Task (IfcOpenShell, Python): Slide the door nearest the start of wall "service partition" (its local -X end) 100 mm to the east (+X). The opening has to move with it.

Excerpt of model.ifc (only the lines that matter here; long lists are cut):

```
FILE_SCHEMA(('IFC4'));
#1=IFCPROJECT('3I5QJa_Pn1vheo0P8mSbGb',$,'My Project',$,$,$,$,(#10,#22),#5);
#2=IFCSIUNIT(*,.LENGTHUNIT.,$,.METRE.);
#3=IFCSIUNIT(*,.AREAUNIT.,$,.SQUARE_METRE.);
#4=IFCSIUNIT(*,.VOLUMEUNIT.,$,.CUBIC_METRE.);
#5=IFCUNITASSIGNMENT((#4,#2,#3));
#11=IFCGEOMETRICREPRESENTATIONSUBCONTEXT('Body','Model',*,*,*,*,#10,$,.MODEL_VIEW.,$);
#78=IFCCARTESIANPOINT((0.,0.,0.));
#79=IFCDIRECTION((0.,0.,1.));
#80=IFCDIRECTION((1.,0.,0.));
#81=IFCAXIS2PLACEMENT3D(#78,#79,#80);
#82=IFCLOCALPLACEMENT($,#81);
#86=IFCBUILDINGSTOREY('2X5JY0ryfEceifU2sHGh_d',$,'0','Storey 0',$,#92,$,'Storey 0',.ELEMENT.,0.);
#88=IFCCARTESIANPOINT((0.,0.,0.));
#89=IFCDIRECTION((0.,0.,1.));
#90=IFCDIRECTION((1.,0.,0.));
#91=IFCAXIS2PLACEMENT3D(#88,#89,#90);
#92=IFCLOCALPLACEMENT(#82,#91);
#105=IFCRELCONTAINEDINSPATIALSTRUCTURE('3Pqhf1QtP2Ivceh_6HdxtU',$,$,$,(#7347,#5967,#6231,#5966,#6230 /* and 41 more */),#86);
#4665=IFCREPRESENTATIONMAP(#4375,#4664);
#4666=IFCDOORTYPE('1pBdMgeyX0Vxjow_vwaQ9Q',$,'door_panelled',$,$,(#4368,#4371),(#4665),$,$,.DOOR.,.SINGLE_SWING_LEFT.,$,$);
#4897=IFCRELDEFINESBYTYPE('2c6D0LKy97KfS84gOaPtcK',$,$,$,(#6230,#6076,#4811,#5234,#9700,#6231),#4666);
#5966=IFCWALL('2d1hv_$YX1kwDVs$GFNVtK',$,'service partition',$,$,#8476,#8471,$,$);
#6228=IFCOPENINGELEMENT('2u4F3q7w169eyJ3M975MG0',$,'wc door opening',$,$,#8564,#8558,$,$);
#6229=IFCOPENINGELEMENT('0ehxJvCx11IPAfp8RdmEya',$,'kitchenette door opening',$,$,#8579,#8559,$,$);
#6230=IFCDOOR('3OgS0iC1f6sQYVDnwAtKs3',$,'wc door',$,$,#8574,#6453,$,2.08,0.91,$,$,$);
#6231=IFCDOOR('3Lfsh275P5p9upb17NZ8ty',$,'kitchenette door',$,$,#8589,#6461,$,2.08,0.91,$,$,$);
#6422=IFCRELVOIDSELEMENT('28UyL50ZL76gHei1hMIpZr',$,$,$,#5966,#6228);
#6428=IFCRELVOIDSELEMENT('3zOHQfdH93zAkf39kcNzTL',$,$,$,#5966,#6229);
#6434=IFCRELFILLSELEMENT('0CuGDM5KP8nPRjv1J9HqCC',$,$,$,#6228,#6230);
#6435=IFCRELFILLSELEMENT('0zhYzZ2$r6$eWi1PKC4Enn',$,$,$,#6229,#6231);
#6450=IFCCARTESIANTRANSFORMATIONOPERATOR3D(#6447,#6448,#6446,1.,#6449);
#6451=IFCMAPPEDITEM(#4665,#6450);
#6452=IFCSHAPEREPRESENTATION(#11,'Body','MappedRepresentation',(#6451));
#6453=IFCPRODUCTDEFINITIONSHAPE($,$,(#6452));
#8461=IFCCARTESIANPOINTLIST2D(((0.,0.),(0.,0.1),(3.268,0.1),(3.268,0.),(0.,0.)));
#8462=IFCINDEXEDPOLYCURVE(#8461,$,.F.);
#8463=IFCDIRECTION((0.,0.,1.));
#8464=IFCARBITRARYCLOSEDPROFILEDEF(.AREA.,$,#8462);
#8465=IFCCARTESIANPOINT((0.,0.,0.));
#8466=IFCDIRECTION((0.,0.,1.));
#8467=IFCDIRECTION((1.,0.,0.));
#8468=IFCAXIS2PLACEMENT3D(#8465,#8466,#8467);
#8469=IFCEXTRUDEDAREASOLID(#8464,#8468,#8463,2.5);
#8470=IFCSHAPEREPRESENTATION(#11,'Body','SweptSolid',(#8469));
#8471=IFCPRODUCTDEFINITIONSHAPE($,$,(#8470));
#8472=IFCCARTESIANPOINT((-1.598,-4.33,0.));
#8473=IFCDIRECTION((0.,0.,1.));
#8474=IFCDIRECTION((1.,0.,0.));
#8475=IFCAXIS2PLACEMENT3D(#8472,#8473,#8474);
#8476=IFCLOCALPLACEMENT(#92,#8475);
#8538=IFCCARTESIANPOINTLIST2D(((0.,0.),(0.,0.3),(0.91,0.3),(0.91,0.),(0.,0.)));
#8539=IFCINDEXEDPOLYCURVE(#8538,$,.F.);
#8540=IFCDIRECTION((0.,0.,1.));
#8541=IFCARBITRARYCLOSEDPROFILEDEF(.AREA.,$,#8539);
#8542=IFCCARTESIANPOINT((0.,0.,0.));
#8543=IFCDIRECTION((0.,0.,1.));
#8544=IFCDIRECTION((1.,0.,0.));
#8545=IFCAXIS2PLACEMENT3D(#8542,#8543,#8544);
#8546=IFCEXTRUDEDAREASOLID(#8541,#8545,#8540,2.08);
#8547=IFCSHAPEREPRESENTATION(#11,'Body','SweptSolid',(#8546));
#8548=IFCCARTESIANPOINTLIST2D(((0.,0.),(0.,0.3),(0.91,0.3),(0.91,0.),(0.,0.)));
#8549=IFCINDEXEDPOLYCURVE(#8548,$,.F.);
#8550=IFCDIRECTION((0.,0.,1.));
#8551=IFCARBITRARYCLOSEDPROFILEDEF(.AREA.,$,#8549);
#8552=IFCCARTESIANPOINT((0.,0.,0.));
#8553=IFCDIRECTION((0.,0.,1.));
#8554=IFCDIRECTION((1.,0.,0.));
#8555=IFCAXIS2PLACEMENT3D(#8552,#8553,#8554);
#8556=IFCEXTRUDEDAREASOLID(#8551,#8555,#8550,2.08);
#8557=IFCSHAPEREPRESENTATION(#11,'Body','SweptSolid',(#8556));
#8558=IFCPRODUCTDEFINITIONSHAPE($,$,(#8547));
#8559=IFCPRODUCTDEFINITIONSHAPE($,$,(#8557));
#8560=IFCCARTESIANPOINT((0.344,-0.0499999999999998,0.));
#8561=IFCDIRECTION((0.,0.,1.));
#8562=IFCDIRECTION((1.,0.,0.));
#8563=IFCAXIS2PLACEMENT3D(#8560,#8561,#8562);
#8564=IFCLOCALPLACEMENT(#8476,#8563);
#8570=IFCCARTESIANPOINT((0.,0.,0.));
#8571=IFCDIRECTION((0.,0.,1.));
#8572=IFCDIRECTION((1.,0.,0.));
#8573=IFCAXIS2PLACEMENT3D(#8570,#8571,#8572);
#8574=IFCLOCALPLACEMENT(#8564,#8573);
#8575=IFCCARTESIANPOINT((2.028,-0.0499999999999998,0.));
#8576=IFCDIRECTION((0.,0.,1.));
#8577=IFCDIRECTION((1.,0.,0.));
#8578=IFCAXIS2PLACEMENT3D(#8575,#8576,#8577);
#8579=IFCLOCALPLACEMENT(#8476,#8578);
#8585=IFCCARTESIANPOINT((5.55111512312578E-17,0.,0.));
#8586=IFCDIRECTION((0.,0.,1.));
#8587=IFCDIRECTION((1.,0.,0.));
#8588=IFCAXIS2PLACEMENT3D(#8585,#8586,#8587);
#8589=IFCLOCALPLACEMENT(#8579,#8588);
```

```python
import ifcopenshell
import ifcopenshell.api.geometry
import ifcopenshell.util.placement
import ifcopenshell.util.unit

model = ifcopenshell.open("model.ifc")
unit_scale = ifcopenshell.util.unit.calculate_unit_scale(model)

door = model.by_guid("3OgS0iC1f6sQYVDnwAtKs3")
opening = door.FillsVoids[0].RelatingOpeningElement
wall = opening.VoidsElements[0].RelatingBuildingElement

wall_matrix = ifcopenshell.util.placement.get_local_placement(wall.ObjectPlacement)
shift = wall_matrix[:3, 0] * 0.1 / unit_scale
before = ifcopenshell.util.placement.get_local_placement(door.ObjectPlacement)[:3, 3].copy()

# The door is placed relative to its opening, so it follows when the opening moves.
matrix = ifcopenshell.util.placement.get_local_placement(opening.ObjectPlacement)
matrix[:3, 3] += shift
ifcopenshell.api.geometry.edit_object_placement(
    model, product=opening, matrix=matrix, is_si=False, should_transform_children=True
)

after = ifcopenshell.util.placement.get_local_placement(door.ObjectPlacement)[:3, 3]
print("door moved by", (after - before).round(3) + 0.0)

model.write("model_edited.ifc")
```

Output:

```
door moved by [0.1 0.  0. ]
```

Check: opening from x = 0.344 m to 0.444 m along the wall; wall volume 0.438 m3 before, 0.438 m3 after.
